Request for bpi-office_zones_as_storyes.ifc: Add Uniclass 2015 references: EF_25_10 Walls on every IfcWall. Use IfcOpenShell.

First a look at what the model holds.

```python
import ifcopenshell

model = ifcopenshell.open("bpi-office_zones_as_storyes.ifc")
print(model.schema)
print("classifications:", [c.Name for c in model.by_type("IfcClassification")])
for ifc_class in ("IfcDoor", "IfcRoof", "IfcStair", "IfcWall", "IfcWindow"):
    print(ifc_class, len(model.by_type(ifc_class)))
```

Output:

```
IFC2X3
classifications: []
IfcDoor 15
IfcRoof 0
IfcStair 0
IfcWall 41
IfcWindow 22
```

```python
import ifcopenshell
import ifcopenshell.api.classification

model = ifcopenshell.open("bpi-office_zones_as_storyes.ifc")

# IFC2X3 requires Source and Edition and has no link from the project to the system.
system = model.create_entity("IfcClassification", Source="NBS", Edition="2015", Name="Uniclass 2015")

codes = {
    "IfcWall": ("EF_25_10", "Walls"),
}
for ifc_class, (code, name) in codes.items():
    products = model.by_type(ifc_class)
    ifcopenshell.api.classification.add_reference(
        model, products=products, classification=system, identification=code, name=name
    )
    print(code, len(products))

model.write("bpi-office_zones_as_storyes_edited.ifc")
```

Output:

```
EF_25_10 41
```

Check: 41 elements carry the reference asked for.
